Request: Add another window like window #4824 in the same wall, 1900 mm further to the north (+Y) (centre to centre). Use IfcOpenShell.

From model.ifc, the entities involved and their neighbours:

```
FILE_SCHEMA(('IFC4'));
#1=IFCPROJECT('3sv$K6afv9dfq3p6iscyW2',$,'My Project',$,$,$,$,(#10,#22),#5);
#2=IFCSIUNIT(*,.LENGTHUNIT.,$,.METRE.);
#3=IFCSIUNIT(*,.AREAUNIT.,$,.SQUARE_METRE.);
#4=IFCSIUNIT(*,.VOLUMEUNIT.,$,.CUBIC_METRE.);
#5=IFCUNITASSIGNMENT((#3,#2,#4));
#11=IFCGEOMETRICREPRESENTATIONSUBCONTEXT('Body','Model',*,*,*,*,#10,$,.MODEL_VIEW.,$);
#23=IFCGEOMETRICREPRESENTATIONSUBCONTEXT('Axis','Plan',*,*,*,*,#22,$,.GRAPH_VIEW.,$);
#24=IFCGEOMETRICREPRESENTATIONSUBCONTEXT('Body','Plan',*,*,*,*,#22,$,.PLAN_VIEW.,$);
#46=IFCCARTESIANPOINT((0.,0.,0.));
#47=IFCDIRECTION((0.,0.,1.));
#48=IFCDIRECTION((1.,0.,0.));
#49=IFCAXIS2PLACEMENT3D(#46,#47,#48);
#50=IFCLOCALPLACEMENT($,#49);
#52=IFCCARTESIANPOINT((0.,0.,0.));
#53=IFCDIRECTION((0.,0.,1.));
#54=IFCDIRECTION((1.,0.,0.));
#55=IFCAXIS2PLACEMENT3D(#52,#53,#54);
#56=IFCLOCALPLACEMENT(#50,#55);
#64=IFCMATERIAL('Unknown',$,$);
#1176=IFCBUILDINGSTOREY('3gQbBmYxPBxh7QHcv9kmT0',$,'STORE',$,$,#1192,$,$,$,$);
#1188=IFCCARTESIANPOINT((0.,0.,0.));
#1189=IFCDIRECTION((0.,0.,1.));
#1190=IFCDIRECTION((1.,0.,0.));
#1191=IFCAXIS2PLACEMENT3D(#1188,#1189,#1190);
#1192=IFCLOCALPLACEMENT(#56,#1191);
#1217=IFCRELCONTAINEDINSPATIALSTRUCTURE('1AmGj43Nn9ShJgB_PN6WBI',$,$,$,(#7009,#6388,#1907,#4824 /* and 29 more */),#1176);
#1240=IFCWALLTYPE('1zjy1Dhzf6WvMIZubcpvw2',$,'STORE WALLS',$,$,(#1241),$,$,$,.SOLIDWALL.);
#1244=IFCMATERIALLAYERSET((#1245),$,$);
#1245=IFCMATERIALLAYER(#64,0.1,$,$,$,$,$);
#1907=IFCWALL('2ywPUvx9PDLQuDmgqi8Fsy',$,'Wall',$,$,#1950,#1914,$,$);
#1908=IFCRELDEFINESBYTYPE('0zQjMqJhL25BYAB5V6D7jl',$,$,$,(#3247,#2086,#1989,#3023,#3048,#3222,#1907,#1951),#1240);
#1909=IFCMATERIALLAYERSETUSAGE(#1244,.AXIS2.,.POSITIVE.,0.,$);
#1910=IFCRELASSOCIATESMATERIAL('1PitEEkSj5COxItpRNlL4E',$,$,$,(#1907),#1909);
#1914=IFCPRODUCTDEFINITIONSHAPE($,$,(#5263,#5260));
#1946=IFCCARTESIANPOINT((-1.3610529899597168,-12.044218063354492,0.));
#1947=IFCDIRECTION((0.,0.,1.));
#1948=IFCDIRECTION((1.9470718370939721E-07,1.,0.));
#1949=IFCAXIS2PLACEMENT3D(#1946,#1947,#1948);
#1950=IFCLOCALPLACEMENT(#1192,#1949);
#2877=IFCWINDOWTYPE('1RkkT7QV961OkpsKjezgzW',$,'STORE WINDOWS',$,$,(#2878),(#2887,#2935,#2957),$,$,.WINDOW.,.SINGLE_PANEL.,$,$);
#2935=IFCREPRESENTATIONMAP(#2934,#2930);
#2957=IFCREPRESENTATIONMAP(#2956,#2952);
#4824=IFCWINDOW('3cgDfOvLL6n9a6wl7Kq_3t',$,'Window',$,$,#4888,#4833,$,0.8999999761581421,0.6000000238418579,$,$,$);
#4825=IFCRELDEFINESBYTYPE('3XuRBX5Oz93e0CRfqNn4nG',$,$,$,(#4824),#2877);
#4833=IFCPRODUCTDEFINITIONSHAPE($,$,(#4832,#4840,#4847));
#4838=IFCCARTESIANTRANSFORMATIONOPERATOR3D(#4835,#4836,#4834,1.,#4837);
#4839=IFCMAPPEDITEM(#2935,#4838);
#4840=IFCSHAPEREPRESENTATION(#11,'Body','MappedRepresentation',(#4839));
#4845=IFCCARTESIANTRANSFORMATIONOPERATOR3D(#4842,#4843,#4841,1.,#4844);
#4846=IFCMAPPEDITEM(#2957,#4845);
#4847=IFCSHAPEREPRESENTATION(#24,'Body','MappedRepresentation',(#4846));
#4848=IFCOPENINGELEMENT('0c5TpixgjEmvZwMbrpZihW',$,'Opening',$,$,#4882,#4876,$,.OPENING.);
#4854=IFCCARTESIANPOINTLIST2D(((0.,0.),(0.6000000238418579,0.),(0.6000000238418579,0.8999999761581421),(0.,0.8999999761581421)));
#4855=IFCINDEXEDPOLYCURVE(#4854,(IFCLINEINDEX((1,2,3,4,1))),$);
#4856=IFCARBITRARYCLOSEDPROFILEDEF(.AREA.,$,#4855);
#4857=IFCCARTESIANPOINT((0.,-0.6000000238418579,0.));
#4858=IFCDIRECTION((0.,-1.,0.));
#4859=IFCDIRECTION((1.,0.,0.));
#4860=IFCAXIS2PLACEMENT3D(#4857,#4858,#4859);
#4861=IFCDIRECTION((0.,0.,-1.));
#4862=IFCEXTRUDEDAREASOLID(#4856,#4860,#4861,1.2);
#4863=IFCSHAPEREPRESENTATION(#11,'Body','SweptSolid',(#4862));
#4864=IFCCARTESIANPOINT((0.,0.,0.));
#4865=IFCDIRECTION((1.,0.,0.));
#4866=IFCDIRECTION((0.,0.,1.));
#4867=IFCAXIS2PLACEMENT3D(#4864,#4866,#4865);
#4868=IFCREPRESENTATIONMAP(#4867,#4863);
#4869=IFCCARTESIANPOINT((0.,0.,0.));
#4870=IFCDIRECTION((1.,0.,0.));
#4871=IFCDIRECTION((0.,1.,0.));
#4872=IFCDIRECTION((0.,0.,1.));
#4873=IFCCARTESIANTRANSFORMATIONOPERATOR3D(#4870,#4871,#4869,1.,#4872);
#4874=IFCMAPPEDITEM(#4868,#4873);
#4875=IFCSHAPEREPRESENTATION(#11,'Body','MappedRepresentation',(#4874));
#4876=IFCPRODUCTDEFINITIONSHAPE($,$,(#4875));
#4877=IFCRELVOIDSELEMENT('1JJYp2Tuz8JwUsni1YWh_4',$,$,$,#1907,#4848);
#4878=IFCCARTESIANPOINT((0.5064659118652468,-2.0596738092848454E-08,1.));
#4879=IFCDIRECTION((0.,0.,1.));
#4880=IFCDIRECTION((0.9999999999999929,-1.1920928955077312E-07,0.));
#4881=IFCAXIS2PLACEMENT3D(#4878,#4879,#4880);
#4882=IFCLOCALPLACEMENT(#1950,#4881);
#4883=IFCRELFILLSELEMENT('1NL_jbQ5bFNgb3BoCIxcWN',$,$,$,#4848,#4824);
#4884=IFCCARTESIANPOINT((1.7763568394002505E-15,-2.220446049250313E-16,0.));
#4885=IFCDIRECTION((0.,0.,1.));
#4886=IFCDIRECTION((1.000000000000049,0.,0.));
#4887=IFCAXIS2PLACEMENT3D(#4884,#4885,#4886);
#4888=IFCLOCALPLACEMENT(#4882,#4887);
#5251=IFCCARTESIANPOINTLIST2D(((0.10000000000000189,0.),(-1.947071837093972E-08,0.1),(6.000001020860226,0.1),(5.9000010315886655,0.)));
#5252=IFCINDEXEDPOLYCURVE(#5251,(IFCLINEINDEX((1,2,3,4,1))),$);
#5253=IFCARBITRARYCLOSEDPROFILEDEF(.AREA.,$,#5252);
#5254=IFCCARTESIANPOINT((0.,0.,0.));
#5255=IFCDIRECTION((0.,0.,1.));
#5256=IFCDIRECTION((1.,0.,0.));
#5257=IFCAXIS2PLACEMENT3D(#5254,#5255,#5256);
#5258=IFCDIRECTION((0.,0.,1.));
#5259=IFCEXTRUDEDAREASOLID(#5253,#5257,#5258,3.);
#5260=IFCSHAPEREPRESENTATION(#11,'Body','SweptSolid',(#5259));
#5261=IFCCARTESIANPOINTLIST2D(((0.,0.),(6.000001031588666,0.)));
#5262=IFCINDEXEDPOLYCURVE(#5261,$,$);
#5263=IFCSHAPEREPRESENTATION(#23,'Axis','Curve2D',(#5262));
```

```python
import ifcopenshell
import ifcopenshell.api.feature
import ifcopenshell.api.geometry
import ifcopenshell.api.root
import ifcopenshell.geom
import ifcopenshell.util.element
import ifcopenshell.util.placement
import ifcopenshell.util.shape
import ifcopenshell.util.unit

model = ifcopenshell.open("model.ifc")
unit_scale = ifcopenshell.util.unit.calculate_unit_scale(model)
settings = ifcopenshell.geom.settings()


def volume(element):
    """Net volume in cubic metres, openings subtracted."""
    shape = ifcopenshell.geom.create_shape(settings, element)
    return ifcopenshell.util.shape.get_volume(shape.geometry)


window = model.by_id(4824)
opening = window.FillsVoids[0].RelatingOpeningElement
wall = opening.VoidsElements[0].RelatingBuildingElement
before = volume(wall)
shift = ifcopenshell.util.placement.get_local_placement(wall.ObjectPlacement)[:3, 0] * 1.9 / unit_scale

# copy_class copies the void relationship, type, container and properties, but no geometry.
new_opening = ifcopenshell.api.root.copy_class(model, product=opening)
new_opening.Representation = ifcopenshell.util.element.copy_deep(
    model, opening.Representation, exclude=["IfcGeometricRepresentationContext", "IfcRepresentationMap"]
)
new_window = ifcopenshell.api.root.copy_class(model, product=window)
new_window.Representation = ifcopenshell.util.element.copy_deep(
    model, window.Representation, exclude=["IfcGeometricRepresentationContext", "IfcRepresentationMap"]
)
ifcopenshell.api.feature.add_filling(model, opening=new_opening, element=new_window)

for old, new in ((opening, new_opening), (window, new_window)):
    matrix = ifcopenshell.util.placement.get_local_placement(old.ObjectPlacement)
    matrix[:3, 3] += shift
    ifcopenshell.api.geometry.edit_object_placement(model, product=new, matrix=matrix, is_si=False)

after = volume(wall)

print(f"wall volume {before:.3f} -> {after:.3f} m3")

model.write("model_rev.ifc")
```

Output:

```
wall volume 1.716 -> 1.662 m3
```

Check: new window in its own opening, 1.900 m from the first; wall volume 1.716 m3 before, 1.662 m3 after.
